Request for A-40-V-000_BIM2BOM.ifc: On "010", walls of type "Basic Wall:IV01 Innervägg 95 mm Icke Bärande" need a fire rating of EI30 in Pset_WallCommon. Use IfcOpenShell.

First a look at what the model holds.

```python
import ifcopenshell
import ifcopenshell.util.element

model = ifcopenshell.open("A-40-V-000_BIM2BOM.ifc")
print(model.schema)
storey = next(s for s in model.by_type("IfcBuildingStorey") if s.Name == "010")
walls = [e for e in ifcopenshell.util.element.get_decomposition(storey) if e.is_a("IfcWall")]
seen = {}
for e in walls:
    element_type = ifcopenshell.util.element.get_type(e)
    key = (element_type.Name if element_type != e and element_type else None, ifcopenshell.util.element.get_pset(e, "Pset_WallCommon", "FireRating"))
    seen[key] = seen.get(key, 0) + 1
for (name, value), count in sorted(seen.items(), key=str):
    print(count, "x", name, "|", value)
```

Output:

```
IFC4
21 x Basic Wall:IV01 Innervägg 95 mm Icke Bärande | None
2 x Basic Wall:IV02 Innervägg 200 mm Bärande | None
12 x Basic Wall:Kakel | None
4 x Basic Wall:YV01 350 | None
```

```python
import ifcopenshell
import ifcopenshell.api.pset
import ifcopenshell.util.element

model = ifcopenshell.open("A-40-V-000_BIM2BOM.ifc")

storey = next(s for s in model.by_type("IfcBuildingStorey") if s.Name == "010")
walls = [e for e in ifcopenshell.util.element.get_decomposition(storey) if e.is_a("IfcWall")]

count = 0
for e in walls:
    element_type = ifcopenshell.util.element.get_type(e)
    if element_type in (None, e) or element_type.Name != "Basic Wall:IV01 Innervägg 95 mm Icke Bärande":
        continue
    # add_pset returns the element's existing set when there is one.
    pset = ifcopenshell.api.pset.add_pset(model, product=e, name="Pset_WallCommon")
    ifcopenshell.api.pset.edit_pset(model, pset=pset, properties={"FireRating": "EI30"})
    count += 1

print(count, "walls updated")

model.write("A-40-V-000_BIM2BOM_updated.ifc")
```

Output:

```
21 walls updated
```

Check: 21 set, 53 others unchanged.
